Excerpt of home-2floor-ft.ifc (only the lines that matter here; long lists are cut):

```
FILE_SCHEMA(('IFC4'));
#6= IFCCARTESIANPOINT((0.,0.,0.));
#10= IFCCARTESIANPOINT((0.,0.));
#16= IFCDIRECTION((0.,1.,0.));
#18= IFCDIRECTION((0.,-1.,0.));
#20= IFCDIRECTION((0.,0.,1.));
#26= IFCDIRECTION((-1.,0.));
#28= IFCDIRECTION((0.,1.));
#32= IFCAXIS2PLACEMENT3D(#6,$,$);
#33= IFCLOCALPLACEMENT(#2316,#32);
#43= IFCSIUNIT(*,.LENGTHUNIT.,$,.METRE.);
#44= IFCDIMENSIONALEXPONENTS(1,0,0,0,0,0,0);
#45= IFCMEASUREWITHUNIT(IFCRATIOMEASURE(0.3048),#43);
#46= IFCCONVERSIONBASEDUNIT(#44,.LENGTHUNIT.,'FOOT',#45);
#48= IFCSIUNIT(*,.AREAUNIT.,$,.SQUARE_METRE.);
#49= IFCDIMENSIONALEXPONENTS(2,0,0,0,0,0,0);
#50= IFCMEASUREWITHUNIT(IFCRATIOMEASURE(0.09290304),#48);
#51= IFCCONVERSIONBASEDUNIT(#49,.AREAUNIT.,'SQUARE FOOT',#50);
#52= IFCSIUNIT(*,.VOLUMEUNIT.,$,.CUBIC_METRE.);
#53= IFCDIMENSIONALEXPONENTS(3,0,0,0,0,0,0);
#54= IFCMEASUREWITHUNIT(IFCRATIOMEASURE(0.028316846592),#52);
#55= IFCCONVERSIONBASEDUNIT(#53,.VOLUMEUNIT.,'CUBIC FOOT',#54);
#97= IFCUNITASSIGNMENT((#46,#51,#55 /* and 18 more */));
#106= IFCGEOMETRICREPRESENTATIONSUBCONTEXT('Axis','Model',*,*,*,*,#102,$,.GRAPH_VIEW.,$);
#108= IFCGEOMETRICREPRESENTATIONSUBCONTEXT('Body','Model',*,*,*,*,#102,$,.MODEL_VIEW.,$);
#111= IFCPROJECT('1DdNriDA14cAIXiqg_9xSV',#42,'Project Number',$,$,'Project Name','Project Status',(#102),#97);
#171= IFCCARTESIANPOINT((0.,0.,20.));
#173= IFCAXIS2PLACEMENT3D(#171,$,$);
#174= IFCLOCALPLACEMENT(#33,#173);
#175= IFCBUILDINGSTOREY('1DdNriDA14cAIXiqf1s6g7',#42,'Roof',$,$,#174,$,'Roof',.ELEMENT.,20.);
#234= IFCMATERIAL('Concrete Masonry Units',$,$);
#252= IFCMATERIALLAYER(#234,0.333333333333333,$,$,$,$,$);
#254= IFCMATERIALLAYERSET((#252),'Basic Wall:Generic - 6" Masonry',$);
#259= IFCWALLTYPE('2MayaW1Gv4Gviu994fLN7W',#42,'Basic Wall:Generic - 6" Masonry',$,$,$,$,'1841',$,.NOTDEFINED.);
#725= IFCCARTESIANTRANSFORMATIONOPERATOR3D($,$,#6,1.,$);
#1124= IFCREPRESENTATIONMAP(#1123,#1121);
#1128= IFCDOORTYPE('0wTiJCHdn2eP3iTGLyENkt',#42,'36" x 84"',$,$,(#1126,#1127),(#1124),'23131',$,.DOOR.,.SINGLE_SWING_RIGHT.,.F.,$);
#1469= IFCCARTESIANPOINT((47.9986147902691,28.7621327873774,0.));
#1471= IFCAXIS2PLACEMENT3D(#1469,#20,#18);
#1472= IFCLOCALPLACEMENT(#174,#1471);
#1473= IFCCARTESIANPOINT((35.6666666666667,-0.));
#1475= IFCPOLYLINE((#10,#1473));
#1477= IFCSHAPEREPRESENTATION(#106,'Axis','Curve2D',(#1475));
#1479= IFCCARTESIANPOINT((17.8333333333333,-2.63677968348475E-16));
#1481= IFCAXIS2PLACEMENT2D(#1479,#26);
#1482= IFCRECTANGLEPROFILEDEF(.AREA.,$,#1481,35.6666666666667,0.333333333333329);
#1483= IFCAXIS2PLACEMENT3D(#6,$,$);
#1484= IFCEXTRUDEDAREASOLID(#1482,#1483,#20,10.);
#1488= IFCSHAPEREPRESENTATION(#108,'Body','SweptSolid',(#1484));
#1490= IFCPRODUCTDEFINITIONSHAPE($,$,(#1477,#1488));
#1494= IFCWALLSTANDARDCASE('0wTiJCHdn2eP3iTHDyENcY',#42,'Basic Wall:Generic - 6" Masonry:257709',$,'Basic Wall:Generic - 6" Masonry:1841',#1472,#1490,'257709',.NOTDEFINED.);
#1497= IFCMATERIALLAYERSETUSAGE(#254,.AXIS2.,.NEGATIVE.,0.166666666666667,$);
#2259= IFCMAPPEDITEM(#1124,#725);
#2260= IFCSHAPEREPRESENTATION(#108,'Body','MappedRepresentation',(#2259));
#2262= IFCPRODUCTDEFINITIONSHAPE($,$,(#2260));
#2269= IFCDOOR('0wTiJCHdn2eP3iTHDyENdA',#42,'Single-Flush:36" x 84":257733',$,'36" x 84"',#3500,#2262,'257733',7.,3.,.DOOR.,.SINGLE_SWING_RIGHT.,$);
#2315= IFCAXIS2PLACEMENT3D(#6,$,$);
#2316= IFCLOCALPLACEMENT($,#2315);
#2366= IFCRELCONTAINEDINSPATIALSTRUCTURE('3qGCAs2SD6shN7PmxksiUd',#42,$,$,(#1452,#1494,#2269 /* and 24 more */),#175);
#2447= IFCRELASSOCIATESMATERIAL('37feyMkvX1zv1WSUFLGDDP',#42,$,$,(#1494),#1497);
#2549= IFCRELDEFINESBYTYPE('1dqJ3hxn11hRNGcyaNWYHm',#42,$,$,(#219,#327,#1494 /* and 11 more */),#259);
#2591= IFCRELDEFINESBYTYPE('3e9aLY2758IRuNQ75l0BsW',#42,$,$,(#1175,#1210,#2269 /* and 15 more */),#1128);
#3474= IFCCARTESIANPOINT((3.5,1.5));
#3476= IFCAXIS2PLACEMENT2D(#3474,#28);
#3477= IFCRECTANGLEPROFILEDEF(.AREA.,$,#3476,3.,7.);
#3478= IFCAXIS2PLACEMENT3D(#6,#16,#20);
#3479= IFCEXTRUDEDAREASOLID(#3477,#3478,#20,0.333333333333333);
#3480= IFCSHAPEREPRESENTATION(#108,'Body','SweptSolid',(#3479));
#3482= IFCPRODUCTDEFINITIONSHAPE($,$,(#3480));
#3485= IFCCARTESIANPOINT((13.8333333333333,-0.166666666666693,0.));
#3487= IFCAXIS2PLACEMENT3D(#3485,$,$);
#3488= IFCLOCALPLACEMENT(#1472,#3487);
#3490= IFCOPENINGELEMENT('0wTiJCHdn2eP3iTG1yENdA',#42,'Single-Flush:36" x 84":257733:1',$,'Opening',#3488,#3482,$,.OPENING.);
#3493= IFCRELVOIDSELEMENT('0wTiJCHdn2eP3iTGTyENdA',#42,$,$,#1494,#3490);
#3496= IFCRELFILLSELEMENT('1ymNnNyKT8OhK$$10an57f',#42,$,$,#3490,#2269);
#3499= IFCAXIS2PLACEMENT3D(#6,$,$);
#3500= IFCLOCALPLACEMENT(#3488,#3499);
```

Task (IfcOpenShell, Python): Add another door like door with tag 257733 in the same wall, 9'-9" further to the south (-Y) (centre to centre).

```python
import ifcopenshell
import ifcopenshell.api.feature
import ifcopenshell.api.geometry
import ifcopenshell.api.root
import ifcopenshell.geom
import ifcopenshell.util.element
import ifcopenshell.util.placement
import ifcopenshell.util.shape
import ifcopenshell.util.unit

model = ifcopenshell.open("home-2floor-ft.ifc")
unit_scale = ifcopenshell.util.unit.calculate_unit_scale(model)
settings = ifcopenshell.geom.settings()


def volume(element):
    """Net volume in cubic metres, openings subtracted."""
    shape = ifcopenshell.geom.create_shape(settings, element)
    return ifcopenshell.util.shape.get_volume(shape.geometry)


def reuse_history(source, copy):
    """copy_class also copies each property set's owner history, people and application; keep the originals."""
    for rel in copy.IsDefinedBy:
        if rel.is_a("IfcRelDefinesByProperties") and (history := rel.RelatingPropertyDefinition.OwnerHistory):
            rel.RelatingPropertyDefinition.OwnerHistory = source.OwnerHistory
            ifcopenshell.util.element.remove_deep2(model, history)


door = model.by_guid("0wTiJCHdn2eP3iTHDyENdA")
opening = door.FillsVoids[0].RelatingOpeningElement
wall = opening.VoidsElements[0].RelatingBuildingElement
before = volume(wall)
shift = ifcopenshell.util.placement.get_local_placement(wall.ObjectPlacement)[:3, 0] * 117 * 0.0254 / unit_scale

# copy_class copies the void relationship, type, container and properties, but no geometry.
new_opening = ifcopenshell.api.root.copy_class(model, product=opening)
new_opening.Representation = ifcopenshell.util.element.copy_deep(
    model, opening.Representation, exclude=["IfcGeometricRepresentationContext", "IfcRepresentationMap"]
)
new_opening.Name = 'Single-Flush:36" x 84"'
new_door = ifcopenshell.api.root.copy_class(model, product=door)
new_door.Representation = ifcopenshell.util.element.copy_deep(
    model, door.Representation, exclude=["IfcGeometricRepresentationContext", "IfcRepresentationMap"]
)
new_door.Name = 'Single-Flush:36" x 84"'
new_door.Tag = None
reuse_history(door, new_door)
ifcopenshell.api.feature.add_filling(model, opening=new_opening, element=new_door)

for old, new in ((opening, new_opening), (door, new_door)):
    matrix = ifcopenshell.util.placement.get_local_placement(old.ObjectPlacement)
    matrix[:3, 3] += shift
    ifcopenshell.api.geometry.edit_object_placement(model, product=new, matrix=matrix, is_si=False)

after = volume(wall)

print(f"wall volume {before:.3f} -> {after:.3f} m3")

model.write("home-2floor-ft_updated.ifc")
```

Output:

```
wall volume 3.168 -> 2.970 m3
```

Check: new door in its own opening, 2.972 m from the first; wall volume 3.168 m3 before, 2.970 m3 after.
